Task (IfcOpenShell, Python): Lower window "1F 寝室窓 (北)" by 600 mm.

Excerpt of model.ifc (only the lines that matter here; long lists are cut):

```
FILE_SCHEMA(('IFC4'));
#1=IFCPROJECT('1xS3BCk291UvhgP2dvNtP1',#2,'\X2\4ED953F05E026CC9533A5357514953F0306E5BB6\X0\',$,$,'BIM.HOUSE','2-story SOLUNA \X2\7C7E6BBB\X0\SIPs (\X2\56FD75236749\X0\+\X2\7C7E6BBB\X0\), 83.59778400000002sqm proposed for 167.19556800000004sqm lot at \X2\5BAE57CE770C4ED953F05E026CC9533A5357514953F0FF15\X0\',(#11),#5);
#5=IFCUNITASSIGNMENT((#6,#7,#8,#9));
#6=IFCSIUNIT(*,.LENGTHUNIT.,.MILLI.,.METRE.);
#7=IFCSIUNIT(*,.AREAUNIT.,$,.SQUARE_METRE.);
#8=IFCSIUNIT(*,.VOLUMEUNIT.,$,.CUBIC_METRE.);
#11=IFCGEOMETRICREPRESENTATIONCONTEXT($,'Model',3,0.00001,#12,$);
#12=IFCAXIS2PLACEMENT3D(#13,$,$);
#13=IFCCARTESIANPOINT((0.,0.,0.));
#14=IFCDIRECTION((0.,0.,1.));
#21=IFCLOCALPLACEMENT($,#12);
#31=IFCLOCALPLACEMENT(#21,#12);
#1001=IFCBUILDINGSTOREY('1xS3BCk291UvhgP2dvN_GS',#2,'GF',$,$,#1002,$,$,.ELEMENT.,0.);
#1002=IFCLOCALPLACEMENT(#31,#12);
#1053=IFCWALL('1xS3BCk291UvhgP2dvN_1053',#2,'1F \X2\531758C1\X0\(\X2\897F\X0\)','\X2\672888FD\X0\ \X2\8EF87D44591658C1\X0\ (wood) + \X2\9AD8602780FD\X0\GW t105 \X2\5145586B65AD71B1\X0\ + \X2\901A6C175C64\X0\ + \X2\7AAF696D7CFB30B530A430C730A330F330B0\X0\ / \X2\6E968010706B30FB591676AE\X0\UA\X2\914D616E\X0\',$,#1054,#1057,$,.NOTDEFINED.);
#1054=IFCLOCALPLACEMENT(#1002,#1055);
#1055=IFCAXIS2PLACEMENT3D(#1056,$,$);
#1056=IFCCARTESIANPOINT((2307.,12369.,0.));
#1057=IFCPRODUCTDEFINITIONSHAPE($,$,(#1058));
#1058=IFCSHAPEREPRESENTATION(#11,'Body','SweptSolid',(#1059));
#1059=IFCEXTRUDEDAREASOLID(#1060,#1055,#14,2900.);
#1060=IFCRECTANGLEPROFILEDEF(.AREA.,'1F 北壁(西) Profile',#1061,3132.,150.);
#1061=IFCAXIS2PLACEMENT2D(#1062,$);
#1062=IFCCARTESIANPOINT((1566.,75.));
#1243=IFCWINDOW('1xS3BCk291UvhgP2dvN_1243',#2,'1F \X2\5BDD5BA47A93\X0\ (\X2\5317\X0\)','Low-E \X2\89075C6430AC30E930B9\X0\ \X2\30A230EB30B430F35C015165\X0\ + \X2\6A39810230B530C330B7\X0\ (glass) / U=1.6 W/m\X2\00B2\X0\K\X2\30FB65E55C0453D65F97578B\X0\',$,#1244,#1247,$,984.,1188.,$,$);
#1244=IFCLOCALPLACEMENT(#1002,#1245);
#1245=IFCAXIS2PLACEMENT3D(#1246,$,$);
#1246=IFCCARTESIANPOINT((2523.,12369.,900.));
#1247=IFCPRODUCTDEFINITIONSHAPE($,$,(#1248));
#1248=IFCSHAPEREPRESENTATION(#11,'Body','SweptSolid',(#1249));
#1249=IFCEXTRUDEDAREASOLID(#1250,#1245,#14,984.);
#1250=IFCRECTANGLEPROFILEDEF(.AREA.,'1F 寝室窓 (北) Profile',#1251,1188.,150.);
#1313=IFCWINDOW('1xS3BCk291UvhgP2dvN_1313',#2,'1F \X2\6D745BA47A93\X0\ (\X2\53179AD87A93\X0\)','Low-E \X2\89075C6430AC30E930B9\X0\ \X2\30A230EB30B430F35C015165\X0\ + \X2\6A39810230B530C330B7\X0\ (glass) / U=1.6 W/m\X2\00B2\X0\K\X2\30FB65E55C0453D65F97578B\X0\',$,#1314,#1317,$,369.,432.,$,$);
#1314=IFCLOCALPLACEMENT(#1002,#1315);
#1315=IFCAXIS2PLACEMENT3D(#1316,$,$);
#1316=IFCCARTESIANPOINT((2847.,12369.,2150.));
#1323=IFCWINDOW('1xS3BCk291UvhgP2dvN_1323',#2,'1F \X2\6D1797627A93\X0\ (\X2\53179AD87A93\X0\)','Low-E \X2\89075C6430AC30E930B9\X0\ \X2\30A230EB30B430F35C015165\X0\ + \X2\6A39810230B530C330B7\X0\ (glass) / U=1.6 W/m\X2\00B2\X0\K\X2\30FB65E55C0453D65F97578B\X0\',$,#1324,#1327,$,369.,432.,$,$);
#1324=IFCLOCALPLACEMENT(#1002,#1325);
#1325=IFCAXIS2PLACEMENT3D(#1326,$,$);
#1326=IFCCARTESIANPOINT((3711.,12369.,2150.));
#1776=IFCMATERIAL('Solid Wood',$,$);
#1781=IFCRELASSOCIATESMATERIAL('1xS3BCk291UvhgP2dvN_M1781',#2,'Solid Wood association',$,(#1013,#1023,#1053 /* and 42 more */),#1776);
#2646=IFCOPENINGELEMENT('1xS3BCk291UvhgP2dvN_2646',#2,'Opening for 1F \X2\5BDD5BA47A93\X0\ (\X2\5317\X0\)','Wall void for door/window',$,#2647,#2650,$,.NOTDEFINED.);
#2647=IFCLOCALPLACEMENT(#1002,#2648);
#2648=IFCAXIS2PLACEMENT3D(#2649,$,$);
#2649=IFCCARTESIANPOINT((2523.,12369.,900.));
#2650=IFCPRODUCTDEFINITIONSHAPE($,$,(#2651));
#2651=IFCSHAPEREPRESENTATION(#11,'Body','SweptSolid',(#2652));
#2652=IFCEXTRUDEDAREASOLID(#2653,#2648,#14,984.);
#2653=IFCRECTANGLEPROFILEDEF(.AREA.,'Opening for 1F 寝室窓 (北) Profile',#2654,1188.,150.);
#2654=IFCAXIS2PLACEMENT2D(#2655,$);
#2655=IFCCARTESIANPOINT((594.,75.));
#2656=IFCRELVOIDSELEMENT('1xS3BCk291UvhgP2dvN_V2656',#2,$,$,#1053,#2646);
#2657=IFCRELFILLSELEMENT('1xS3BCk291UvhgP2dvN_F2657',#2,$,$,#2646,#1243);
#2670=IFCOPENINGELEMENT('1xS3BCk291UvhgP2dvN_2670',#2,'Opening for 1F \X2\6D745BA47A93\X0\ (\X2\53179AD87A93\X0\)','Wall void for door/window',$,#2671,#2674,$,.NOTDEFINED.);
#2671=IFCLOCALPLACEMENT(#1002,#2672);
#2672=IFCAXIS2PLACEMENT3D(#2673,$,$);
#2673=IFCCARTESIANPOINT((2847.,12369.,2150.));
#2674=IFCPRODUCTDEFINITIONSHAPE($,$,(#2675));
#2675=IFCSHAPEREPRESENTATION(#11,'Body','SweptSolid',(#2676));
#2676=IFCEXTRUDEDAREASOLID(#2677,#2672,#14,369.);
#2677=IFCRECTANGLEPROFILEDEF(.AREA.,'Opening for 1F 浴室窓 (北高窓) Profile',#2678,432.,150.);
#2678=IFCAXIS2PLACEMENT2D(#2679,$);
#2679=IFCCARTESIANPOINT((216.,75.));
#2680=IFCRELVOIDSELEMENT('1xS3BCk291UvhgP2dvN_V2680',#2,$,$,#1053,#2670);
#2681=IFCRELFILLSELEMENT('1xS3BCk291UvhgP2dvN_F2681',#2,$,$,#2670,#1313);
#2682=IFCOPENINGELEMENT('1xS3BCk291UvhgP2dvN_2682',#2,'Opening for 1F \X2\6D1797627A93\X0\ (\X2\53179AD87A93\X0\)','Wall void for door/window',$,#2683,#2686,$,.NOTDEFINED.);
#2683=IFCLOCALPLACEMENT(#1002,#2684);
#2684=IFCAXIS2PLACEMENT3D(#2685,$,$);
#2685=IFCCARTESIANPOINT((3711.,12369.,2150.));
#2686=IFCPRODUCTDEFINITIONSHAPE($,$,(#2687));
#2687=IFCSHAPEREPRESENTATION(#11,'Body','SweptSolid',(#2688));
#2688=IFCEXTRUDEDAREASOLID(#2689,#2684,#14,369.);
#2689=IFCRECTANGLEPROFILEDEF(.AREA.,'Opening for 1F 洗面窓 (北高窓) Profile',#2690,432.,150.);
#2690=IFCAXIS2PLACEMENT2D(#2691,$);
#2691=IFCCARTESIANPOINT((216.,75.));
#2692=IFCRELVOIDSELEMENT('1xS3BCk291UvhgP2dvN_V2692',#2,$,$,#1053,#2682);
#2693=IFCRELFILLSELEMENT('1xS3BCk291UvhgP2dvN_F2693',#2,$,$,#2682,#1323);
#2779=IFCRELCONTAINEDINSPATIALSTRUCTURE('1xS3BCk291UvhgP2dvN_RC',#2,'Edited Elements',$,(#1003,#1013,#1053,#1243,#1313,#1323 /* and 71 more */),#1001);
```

```python
import numpy as np
import ifcopenshell
import ifcopenshell.api.geometry
import ifcopenshell.util.placement
import ifcopenshell.util.unit

model = ifcopenshell.open("model.ifc")
unit_scale = ifcopenshell.util.unit.calculate_unit_scale(model)

window = model.by_guid("1xS3BCk291UvhgP2dvN_1243")
opening = window.FillsVoids[0].RelatingOpeningElement
dz = -0.6 / unit_scale

shift = np.array([0.0, 0.0, dz])
# The window is not placed relative to its opening, so move both.
for product in (opening, window):
    matrix = ifcopenshell.util.placement.get_local_placement(product.ObjectPlacement)
    matrix[:3, 3] += shift
    ifcopenshell.api.geometry.edit_object_placement(model, product=product, matrix=matrix, is_si=False)

print(f"moved by {dz * unit_scale:+.3f} m")

model.write("model_edited.ifc")
```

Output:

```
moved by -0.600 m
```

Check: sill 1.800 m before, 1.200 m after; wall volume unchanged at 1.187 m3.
